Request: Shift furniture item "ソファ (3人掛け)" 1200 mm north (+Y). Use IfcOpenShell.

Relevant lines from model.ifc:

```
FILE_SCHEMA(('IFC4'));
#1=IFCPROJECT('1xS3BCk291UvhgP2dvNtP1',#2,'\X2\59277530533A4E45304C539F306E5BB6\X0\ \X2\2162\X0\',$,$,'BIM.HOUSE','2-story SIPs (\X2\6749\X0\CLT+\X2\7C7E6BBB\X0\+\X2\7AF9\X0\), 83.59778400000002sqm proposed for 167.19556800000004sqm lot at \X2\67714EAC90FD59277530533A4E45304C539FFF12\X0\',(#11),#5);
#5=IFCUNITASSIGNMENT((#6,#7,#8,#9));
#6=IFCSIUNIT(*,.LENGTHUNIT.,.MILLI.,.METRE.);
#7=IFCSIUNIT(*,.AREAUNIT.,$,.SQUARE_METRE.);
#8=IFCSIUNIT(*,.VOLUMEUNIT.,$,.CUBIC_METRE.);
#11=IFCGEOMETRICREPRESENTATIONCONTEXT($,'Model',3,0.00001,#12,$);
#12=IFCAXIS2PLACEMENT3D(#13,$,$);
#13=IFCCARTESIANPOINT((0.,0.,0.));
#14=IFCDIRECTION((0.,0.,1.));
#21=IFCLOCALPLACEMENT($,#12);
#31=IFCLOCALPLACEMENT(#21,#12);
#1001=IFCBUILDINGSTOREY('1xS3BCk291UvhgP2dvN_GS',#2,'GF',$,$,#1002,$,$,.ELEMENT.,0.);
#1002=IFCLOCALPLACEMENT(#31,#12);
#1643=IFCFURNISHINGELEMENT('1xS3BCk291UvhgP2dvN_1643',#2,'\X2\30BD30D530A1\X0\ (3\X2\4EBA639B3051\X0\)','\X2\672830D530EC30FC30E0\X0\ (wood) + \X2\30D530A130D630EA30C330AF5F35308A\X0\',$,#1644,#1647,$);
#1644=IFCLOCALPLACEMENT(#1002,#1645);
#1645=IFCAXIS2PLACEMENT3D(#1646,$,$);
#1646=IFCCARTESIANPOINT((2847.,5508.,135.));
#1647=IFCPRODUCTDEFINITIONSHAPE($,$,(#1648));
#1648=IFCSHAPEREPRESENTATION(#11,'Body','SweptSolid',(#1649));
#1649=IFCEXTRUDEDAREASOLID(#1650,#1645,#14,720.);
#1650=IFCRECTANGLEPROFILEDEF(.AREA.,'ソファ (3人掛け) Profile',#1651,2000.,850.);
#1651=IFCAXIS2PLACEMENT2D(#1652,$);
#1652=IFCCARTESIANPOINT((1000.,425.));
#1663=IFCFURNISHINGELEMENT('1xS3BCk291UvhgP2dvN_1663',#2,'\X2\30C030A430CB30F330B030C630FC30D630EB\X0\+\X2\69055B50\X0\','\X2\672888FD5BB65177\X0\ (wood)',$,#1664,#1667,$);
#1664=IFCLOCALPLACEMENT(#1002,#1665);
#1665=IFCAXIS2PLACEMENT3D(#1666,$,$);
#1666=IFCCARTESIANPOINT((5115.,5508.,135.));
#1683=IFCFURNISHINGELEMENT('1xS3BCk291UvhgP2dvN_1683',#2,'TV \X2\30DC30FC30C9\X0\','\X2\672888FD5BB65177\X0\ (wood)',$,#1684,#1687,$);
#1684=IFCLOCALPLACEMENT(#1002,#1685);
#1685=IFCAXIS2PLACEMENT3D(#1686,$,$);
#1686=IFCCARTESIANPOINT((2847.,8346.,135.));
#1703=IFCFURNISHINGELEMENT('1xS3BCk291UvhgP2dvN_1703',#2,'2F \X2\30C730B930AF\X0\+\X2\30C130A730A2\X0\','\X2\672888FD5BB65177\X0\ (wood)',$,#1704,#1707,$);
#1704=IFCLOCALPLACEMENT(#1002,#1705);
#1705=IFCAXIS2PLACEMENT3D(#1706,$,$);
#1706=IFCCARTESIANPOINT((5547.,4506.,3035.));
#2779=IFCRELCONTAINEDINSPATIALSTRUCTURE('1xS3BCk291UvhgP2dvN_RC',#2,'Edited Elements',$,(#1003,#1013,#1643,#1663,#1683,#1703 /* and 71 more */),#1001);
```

```python
import ifcopenshell
import ifcopenshell.api.geometry
import ifcopenshell.util.placement
import ifcopenshell.util.unit

model = ifcopenshell.open("model.ifc")
unit_scale = ifcopenshell.util.unit.calculate_unit_scale(model)

item = model.by_id(1643)
matrix = ifcopenshell.util.placement.get_local_placement(item.ObjectPlacement)
matrix[1, 3] += 1.2 / unit_scale
ifcopenshell.api.geometry.edit_object_placement(model, product=item, matrix=matrix, is_si=False)

print(ifcopenshell.util.placement.get_local_placement(item.ObjectPlacement).round(3) + 0.0)

model.write("model_rev.ifc")
```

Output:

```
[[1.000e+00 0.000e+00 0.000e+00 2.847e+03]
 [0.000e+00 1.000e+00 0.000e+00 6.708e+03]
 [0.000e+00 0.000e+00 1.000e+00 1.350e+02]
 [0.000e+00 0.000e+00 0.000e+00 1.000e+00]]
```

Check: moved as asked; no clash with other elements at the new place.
